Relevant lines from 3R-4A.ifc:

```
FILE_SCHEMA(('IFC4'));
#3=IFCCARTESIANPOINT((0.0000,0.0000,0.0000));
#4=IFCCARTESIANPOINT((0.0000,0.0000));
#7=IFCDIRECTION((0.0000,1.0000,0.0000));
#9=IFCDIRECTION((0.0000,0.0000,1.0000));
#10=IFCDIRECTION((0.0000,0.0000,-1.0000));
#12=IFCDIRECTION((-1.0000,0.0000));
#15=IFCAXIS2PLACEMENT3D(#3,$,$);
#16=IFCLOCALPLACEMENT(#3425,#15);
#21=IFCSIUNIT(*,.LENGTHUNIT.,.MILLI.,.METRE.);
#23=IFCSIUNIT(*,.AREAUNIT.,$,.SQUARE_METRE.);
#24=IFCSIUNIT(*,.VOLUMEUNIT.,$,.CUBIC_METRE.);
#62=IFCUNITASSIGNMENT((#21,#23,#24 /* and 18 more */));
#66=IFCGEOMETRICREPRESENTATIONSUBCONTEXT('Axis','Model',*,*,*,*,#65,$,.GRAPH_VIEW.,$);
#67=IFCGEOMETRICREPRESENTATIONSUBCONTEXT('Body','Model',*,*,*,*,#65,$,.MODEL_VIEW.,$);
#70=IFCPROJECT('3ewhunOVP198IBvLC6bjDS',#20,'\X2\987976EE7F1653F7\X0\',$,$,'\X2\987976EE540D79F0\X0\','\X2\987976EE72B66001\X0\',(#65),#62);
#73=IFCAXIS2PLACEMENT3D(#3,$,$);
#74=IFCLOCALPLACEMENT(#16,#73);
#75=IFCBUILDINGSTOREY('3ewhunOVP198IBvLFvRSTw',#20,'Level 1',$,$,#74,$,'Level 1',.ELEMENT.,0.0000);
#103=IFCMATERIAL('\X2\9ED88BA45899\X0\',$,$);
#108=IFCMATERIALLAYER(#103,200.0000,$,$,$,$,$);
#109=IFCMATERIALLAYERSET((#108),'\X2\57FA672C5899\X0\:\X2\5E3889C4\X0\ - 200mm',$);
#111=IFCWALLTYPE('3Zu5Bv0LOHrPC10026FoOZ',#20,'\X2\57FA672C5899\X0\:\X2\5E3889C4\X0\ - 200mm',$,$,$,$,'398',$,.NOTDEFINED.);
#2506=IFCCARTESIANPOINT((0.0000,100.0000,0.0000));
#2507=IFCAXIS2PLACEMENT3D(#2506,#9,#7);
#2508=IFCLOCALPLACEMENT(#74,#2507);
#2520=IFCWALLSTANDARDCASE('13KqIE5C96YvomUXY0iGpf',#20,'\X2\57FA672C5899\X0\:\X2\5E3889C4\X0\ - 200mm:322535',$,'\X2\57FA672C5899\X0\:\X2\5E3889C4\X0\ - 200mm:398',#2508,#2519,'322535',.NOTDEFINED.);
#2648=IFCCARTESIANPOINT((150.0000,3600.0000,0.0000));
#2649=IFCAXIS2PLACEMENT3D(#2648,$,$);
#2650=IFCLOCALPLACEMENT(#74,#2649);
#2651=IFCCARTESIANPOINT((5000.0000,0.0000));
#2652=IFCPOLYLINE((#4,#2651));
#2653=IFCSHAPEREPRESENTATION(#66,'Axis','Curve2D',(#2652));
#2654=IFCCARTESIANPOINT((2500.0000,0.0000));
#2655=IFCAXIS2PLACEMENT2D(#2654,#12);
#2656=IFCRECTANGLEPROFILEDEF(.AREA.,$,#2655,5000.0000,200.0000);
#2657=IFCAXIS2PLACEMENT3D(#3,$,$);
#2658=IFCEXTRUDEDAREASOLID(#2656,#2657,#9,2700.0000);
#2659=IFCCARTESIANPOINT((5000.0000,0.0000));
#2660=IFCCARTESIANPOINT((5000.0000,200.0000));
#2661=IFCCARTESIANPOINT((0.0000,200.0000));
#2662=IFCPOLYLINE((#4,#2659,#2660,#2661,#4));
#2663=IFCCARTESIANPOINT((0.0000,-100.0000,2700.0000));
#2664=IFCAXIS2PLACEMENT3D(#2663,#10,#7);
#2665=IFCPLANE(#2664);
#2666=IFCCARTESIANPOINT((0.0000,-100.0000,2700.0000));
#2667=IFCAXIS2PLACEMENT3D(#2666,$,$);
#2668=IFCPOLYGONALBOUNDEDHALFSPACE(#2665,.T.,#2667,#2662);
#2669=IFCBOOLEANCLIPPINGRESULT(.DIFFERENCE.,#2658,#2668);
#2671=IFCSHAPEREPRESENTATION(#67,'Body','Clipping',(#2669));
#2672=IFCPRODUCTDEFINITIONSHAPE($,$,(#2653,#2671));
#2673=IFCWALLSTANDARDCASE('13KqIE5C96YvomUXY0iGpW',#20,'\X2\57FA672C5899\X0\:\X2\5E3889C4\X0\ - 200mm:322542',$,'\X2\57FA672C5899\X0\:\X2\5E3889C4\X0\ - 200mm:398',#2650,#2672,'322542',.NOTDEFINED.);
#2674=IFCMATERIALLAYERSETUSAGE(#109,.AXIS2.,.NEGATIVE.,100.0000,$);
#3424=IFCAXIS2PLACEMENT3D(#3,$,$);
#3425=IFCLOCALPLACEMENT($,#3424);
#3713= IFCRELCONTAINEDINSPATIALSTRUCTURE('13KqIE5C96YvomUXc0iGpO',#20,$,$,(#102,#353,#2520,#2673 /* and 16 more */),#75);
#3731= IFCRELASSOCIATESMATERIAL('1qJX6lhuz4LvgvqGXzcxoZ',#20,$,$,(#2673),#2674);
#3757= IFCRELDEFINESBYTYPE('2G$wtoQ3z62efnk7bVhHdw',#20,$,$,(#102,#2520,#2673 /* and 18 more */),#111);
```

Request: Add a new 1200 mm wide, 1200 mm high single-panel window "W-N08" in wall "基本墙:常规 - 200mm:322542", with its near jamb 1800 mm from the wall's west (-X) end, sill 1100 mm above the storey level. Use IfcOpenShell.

```python
import numpy as np
import ifcopenshell
import ifcopenshell.api.feature
import ifcopenshell.api.geometry
import ifcopenshell.api.root
import ifcopenshell.api.spatial
import ifcopenshell.geom
import ifcopenshell.util.element
import ifcopenshell.util.placement
import ifcopenshell.util.representation
import ifcopenshell.util.shape
import ifcopenshell.util.unit

model = ifcopenshell.open("3R-4A.ifc")
unit_scale = ifcopenshell.util.unit.calculate_unit_scale(model)
settings = ifcopenshell.geom.settings()


def volume(element):
    """Net volume in cubic metres, openings subtracted."""
    shape = ifcopenshell.geom.create_shape(settings, element)
    return ifcopenshell.util.shape.get_volume(shape.geometry)


wall = model.by_guid("13KqIE5C96YvomUXY0iGpW")
storey = ifcopenshell.util.element.get_container(wall, ifc_class="IfcBuildingStorey")
context = ifcopenshell.util.representation.get_context(model, "Model", "Body", "MODEL_VIEW")
before = volume(wall)

width, height, from_end, sill = 1.2, 1.2, 1.8, 1.1  # metres

# The wall runs along its own X axis, and the end named is its -X end.
wall_shape = ifcopenshell.geom.create_shape(settings, wall)
x, y, z = ifcopenshell.util.shape.get_vertices(wall_shape.geometry).T
start = x.min() + from_end
face, thickness = float(y.min()), float(y.max() - y.min())
wall_matrix = ifcopenshell.util.placement.get_local_placement(wall.ObjectPlacement)
level = ifcopenshell.util.placement.get_local_placement(storey.ObjectPlacement)[2, 3]


def in_wall(x, y):
    """Placement at x, y metres in the wall's axes, at sill height."""
    matrix = wall_matrix.copy()
    matrix[:, 3] = wall_matrix @ np.array([x / unit_scale, y / unit_scale, 0.0, 1.0])
    matrix[2, 3] = level + sill / unit_scale
    return matrix


# Opening: a box that overshoots both wall faces by 50 mm.
opening = ifcopenshell.api.root.create_entity(model, ifc_class="IfcOpeningElement", predefined_type="OPENING")
box = ifcopenshell.api.geometry.add_wall_representation(
    model, context=context, length=width, height=height, thickness=thickness + 0.1
)
ifcopenshell.api.geometry.assign_representation(model, product=opening, representation=box)
ifcopenshell.api.geometry.edit_object_placement(model, product=opening, matrix=in_wall(start, face - 0.05), is_si=False)
ifcopenshell.api.feature.add_feature(model, feature=opening, element=wall)

window = ifcopenshell.api.root.create_entity(model, ifc_class="IfcWindow", name="W-N08", predefined_type="WINDOW")
window.OverallWidth, window.OverallHeight = width / unit_scale, height / unit_scale
window.PartitioningType = "SINGLE_PANEL"
body = ifcopenshell.api.geometry.add_window_representation(
    model,
    context=context,
    overall_width=window.OverallWidth,
    overall_height=window.OverallHeight,
    partition_type="SINGLE_PANEL",
)
ifcopenshell.api.geometry.assign_representation(model, product=window, representation=body)
ifcopenshell.api.spatial.assign_container(model, products=[window], relating_structure=storey)
ifcopenshell.api.feature.add_filling(model, opening=opening, element=window)

# Centre the window in the wall's thickness.
ifcopenshell.api.geometry.edit_object_placement(model, product=window, matrix=in_wall(start, face), is_si=False)
window_shape = ifcopenshell.geom.create_shape(settings, window)
depth = ifcopenshell.util.shape.get_vertices(window_shape.geometry)[:, 1]
offset = face + thickness / 2 - (depth.min() + depth.max()) / 2
ifcopenshell.api.geometry.edit_object_placement(model, product=window, matrix=in_wall(start, offset), is_si=False)

after = volume(wall)

print(f"wall volume {before:.3f} -> {after:.3f} m3")

model.write("3R-4A_edited.ifc")
```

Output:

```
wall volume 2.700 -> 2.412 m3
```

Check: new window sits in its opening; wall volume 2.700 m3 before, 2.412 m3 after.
